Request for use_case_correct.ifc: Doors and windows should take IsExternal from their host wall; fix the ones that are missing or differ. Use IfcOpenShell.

First a look at what the model holds.

```python
import ifcopenshell
import ifcopenshell.util.element

model = ifcopenshell.open("use_case_correct.ifc")
print(model.schema)
seen = {}
for e in model.by_type("IfcDoor") + model.by_type("IfcWindow"):
    if not e.FillsVoids:
        continue
    host = e.FillsVoids[0].RelatingOpeningElement.VoidsElements[0].RelatingBuildingElement
    own = ifcopenshell.util.element.get_pset(e, f"Pset_{e.is_a()[3:].removesuffix('StandardCase')}Common", "IsExternal")
    wall = ifcopenshell.util.element.get_pset(host, "Pset_WallCommon", "IsExternal")
    seen[e.is_a(), own, wall] = seen.get((e.is_a(), own, wall), 0) + 1
for (cls, own, wall), count in sorted(seen.items(), key=str):
    print(count, cls, "IsExternal:", own, "| host wall:", wall)
```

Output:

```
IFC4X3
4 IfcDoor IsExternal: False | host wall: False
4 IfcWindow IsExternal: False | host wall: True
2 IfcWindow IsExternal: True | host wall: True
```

```python
import ifcopenshell
import ifcopenshell.api.pset
import ifcopenshell.util.element

model = ifcopenshell.open("use_case_correct.ifc")

count = 0
for ifc_class, pset_name in (("IfcDoor", "Pset_DoorCommon"), ("IfcWindow", "Pset_WindowCommon")):
    for e in model.by_type(ifc_class):
        if not e.FillsVoids:
            continue
        host = e.FillsVoids[0].RelatingOpeningElement.VoidsElements[0].RelatingBuildingElement
        external = ifcopenshell.util.element.get_pset(host, "Pset_WallCommon", "IsExternal")
        if external is None or ifcopenshell.util.element.get_pset(e, pset_name, "IsExternal") == external:
            continue
        pset = ifcopenshell.api.pset.add_pset(model, product=e, name=pset_name)
        ifcopenshell.api.pset.edit_pset(model, pset=pset, properties={"IsExternal": external})
        count += 1

print(count, "updated")

model.write("use_case_correct_edited.ifc")
```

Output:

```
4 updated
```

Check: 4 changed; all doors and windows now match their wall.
